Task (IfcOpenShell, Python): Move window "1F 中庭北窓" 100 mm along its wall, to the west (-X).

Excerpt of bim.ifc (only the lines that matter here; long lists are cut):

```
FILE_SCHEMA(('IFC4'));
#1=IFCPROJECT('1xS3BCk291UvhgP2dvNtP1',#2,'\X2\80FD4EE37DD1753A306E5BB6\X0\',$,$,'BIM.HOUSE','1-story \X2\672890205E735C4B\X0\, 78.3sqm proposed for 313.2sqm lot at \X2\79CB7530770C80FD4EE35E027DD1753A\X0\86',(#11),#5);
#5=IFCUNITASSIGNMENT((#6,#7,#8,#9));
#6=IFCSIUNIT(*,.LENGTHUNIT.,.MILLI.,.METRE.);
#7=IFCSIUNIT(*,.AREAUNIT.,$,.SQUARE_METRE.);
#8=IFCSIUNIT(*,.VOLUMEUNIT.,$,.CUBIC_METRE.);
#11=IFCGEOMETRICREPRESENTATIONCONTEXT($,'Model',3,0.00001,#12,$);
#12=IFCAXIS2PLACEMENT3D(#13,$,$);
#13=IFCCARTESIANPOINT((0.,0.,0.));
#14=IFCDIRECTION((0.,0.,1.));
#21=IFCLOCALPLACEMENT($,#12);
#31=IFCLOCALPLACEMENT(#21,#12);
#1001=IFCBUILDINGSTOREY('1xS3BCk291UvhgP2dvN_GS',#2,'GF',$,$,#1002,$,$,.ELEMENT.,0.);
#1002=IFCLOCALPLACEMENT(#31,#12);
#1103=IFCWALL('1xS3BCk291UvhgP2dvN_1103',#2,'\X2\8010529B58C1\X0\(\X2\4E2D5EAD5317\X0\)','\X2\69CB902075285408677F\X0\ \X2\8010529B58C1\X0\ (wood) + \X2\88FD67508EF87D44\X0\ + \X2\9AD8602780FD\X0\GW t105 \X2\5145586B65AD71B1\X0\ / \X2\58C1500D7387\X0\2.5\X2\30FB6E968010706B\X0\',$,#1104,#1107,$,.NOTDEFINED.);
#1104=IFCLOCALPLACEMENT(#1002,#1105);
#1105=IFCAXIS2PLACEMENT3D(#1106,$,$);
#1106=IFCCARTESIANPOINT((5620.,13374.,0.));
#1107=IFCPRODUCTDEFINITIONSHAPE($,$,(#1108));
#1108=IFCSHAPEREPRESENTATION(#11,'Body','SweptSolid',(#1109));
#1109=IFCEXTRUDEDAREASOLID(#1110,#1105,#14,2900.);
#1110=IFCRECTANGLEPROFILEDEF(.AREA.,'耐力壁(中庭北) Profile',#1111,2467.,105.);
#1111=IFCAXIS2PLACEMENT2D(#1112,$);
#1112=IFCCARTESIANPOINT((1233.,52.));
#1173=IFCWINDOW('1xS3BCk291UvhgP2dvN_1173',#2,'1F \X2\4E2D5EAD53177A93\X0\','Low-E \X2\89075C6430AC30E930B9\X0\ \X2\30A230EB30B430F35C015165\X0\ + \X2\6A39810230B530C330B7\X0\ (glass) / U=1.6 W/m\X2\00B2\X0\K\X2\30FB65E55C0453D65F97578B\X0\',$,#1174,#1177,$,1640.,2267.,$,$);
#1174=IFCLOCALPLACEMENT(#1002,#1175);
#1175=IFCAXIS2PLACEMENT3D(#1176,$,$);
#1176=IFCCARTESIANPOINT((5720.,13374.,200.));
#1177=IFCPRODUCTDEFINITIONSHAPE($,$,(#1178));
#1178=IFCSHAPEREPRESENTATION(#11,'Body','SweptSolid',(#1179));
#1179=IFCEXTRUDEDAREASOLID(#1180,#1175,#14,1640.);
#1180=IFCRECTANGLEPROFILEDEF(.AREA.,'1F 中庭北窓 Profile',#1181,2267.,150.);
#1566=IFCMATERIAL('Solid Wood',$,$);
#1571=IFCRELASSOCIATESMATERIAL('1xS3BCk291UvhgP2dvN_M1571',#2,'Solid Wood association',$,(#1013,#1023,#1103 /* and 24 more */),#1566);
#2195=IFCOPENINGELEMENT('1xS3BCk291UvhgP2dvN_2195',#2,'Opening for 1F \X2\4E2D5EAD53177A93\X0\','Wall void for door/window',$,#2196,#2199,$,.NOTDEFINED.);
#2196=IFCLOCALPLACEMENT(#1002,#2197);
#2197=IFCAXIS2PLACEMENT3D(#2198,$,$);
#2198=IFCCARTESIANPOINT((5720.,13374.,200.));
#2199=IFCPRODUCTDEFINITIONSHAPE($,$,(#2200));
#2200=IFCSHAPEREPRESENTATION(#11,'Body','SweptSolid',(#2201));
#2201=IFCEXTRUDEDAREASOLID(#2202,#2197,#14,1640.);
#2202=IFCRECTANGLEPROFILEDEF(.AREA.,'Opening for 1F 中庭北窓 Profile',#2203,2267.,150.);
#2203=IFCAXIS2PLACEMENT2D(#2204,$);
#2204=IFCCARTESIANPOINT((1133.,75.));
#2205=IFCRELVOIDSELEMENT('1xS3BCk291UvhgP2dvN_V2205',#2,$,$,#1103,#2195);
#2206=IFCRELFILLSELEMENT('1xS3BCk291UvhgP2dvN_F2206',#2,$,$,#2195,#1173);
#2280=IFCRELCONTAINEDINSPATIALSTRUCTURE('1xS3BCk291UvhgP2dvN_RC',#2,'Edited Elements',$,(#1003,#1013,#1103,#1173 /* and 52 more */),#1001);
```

```python
import ifcopenshell
import ifcopenshell.api.geometry
import ifcopenshell.util.placement

model = ifcopenshell.open("bim.ifc")

window = model.by_guid("1xS3BCk291UvhgP2dvN_1173")
opening = window.FillsVoids[0].RelatingOpeningElement
wall = opening.VoidsElements[0].RelatingBuildingElement

wall_matrix = ifcopenshell.util.placement.get_local_placement(wall.ObjectPlacement)
shift = wall_matrix[:3, 0] * -100.0
before = ifcopenshell.util.placement.get_local_placement(window.ObjectPlacement)[:3, 3].copy()

# The window is not placed relative to its opening, so move both.
for product in (opening, window):
    matrix = ifcopenshell.util.placement.get_local_placement(product.ObjectPlacement)
    matrix[:3, 3] += shift
    ifcopenshell.api.geometry.edit_object_placement(model, product=product, matrix=matrix, is_si=False)

after = ifcopenshell.util.placement.get_local_placement(window.ObjectPlacement)[:3, 3]
print("window moved by", (after - before).round(3) + 0.0)

model.write("bim_rev.ifc")
```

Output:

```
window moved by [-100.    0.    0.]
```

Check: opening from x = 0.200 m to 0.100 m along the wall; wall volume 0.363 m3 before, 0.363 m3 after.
